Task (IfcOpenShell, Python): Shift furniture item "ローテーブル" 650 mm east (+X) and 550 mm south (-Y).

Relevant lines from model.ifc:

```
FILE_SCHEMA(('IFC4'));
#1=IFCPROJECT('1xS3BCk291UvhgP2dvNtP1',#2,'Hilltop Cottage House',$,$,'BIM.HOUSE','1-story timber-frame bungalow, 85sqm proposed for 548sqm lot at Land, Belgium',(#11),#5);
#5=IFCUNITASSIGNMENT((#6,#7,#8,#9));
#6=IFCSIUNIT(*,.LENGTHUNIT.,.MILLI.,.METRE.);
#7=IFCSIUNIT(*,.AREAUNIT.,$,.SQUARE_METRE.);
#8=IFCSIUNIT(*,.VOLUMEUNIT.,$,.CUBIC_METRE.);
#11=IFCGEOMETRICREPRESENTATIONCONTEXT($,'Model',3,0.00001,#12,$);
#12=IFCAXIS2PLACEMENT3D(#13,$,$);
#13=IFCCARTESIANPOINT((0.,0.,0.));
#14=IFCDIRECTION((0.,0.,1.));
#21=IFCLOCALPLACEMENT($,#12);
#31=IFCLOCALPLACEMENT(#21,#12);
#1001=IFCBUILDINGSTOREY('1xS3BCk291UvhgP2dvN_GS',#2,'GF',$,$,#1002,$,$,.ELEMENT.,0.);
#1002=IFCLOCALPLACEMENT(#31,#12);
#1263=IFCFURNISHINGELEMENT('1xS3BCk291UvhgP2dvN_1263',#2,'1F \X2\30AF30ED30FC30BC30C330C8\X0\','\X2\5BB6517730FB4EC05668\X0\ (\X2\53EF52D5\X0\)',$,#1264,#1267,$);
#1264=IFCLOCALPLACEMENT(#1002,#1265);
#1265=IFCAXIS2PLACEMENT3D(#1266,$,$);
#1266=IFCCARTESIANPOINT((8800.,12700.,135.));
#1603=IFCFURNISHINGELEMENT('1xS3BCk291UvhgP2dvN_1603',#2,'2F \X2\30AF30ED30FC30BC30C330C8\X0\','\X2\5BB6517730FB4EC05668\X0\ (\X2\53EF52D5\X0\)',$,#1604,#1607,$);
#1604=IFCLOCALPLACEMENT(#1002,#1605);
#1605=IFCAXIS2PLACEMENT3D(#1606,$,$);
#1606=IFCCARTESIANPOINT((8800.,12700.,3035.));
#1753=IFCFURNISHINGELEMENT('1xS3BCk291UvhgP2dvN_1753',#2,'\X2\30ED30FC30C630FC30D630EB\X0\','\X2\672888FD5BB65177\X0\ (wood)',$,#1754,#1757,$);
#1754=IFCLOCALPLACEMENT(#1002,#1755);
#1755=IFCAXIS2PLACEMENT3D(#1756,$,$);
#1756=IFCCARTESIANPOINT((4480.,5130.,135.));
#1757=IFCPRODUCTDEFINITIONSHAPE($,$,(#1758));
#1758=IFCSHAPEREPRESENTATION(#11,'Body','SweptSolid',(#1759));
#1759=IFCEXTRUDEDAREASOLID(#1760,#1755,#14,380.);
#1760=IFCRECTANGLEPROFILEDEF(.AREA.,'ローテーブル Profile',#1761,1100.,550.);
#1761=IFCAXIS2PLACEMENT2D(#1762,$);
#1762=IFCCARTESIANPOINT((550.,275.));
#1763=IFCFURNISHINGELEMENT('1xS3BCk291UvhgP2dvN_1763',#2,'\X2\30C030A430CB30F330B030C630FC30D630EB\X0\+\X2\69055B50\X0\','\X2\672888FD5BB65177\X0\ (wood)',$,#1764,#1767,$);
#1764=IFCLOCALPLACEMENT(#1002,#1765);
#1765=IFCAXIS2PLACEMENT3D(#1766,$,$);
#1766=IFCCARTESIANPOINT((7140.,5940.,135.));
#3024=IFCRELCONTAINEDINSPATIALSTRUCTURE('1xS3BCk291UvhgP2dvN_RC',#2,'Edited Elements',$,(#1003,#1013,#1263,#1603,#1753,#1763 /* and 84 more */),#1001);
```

```python
import ifcopenshell
import ifcopenshell.api.geometry
import ifcopenshell.util.placement
import ifcopenshell.util.unit

model = ifcopenshell.open("model.ifc")
unit_scale = ifcopenshell.util.unit.calculate_unit_scale(model)

item = model.by_guid("1xS3BCk291UvhgP2dvN_1753")
matrix = ifcopenshell.util.placement.get_local_placement(item.ObjectPlacement)
matrix[0, 3] += 0.65 / unit_scale
matrix[1, 3] -= 0.55 / unit_scale
ifcopenshell.api.geometry.edit_object_placement(model, product=item, matrix=matrix, is_si=False)

print(ifcopenshell.util.placement.get_local_placement(item.ObjectPlacement).round(3) + 0.0)

model.write("model_updated.ifc")
```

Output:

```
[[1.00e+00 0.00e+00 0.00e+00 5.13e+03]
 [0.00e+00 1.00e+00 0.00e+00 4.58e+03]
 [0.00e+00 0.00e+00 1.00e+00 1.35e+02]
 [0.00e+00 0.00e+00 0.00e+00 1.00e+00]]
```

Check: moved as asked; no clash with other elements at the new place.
